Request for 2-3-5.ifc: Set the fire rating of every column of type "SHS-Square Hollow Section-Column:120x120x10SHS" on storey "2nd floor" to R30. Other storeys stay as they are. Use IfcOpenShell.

First a look at what the model holds.

```python
import ifcopenshell
import ifcopenshell.util.element

model = ifcopenshell.open("2-3-5.ifc")
print(model.schema)
storey = next(s for s in model.by_type("IfcBuildingStorey") if s.Name == "2nd floor")
columns = [e for e in ifcopenshell.util.element.get_decomposition(storey) if e.is_a("IfcColumn")]
seen = {}
for e in columns:
    element_type = ifcopenshell.util.element.get_type(e)
    key = (element_type.Name if element_type != e and element_type else None, ifcopenshell.util.element.get_pset(e, "Pset_ColumnCommon", "FireRating"))
    seen[key] = seen.get(key, 0) + 1
for (name, value), count in sorted(seen.items(), key=str):
    print(count, "x", name, "|", value)
```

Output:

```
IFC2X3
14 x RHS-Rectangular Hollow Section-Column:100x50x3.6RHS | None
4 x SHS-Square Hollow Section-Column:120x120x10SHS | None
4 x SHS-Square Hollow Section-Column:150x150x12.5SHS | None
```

```python
import ifcopenshell
import ifcopenshell.api.pset
import ifcopenshell.util.element

model = ifcopenshell.open("2-3-5.ifc")

storey = next(s for s in model.by_type("IfcBuildingStorey") if s.Name == "2nd floor")
columns = [e for e in ifcopenshell.util.element.get_decomposition(storey) if e.is_a("IfcColumn")]

count = 0
for e in columns:
    element_type = ifcopenshell.util.element.get_type(e)
    if element_type in (None, e) or element_type.Name != "SHS-Square Hollow Section-Column:120x120x10SHS":
        continue
    # add_pset returns the element's existing set when there is one.
    pset = ifcopenshell.api.pset.add_pset(model, product=e, name="Pset_ColumnCommon")
    ifcopenshell.api.pset.edit_pset(model, pset=pset, properties={"FireRating": "R30"})
    count += 1

print(count, "columns updated")

model.write("2-3-5_v2.ifc")
```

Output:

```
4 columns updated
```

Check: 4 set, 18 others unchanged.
